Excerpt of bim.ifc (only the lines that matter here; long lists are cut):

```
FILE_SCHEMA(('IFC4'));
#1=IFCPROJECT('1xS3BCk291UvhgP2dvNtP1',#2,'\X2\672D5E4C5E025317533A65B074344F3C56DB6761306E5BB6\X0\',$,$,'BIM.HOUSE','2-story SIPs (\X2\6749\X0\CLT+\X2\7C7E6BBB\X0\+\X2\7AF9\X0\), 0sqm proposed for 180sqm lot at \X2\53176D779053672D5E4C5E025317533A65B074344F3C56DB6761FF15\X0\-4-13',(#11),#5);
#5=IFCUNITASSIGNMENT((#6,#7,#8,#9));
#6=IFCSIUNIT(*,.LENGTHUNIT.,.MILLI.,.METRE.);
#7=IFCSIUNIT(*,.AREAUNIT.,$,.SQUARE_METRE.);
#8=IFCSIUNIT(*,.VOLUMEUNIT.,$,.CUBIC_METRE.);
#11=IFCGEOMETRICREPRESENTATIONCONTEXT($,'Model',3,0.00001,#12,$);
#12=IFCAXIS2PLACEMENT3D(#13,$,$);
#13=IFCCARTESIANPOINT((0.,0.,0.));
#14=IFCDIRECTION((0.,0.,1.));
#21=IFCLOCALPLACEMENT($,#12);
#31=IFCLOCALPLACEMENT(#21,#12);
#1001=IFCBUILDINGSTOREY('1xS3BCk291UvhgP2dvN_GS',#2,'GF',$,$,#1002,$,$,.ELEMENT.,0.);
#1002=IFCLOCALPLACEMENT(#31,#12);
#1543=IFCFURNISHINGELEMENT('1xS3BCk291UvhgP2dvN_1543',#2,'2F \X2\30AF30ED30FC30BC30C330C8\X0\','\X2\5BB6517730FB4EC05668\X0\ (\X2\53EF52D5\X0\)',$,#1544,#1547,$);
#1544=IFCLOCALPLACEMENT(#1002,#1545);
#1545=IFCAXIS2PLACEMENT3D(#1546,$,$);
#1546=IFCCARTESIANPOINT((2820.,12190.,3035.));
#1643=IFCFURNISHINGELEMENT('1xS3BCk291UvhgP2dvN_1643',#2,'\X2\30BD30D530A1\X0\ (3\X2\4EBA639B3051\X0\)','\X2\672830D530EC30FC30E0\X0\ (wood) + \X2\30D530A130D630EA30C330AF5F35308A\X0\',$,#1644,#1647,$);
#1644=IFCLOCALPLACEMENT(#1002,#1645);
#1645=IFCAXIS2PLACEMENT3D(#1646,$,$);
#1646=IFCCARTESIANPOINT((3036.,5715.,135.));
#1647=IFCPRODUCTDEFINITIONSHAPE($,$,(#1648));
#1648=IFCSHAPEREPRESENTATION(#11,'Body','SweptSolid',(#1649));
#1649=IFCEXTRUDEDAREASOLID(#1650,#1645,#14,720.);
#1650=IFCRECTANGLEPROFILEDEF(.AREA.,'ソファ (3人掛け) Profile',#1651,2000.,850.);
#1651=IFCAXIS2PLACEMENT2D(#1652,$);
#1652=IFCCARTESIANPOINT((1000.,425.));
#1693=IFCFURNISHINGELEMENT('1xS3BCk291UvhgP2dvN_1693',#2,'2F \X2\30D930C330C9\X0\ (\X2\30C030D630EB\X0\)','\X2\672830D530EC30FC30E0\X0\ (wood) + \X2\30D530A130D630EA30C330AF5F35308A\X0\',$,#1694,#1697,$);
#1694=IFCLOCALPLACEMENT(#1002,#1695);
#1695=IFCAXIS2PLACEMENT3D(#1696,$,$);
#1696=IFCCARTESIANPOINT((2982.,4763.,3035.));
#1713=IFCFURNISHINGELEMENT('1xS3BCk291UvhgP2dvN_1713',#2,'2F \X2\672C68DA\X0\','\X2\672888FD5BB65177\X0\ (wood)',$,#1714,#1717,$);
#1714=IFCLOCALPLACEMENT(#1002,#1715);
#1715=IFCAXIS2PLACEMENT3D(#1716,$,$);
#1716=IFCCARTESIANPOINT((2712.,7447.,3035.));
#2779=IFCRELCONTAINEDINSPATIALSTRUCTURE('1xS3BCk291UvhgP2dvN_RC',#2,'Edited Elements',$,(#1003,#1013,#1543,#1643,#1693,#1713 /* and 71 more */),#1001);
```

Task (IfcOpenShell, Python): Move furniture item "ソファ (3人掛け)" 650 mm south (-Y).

```python
import ifcopenshell
import ifcopenshell.api.geometry
import ifcopenshell.util.placement

model = ifcopenshell.open("bim.ifc")

item = model.by_guid("1xS3BCk291UvhgP2dvN_1643")
matrix = ifcopenshell.util.placement.get_local_placement(item.ObjectPlacement)
matrix[1, 3] -= 650.0
ifcopenshell.api.geometry.edit_object_placement(model, product=item, matrix=matrix, is_si=False)

print(ifcopenshell.util.placement.get_local_placement(item.ObjectPlacement).round(3) + 0.0)

model.write("bim_updated.ifc")
```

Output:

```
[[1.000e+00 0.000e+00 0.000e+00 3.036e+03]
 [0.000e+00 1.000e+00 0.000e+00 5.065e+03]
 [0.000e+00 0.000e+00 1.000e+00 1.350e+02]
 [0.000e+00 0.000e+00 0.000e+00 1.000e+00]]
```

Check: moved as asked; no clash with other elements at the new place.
